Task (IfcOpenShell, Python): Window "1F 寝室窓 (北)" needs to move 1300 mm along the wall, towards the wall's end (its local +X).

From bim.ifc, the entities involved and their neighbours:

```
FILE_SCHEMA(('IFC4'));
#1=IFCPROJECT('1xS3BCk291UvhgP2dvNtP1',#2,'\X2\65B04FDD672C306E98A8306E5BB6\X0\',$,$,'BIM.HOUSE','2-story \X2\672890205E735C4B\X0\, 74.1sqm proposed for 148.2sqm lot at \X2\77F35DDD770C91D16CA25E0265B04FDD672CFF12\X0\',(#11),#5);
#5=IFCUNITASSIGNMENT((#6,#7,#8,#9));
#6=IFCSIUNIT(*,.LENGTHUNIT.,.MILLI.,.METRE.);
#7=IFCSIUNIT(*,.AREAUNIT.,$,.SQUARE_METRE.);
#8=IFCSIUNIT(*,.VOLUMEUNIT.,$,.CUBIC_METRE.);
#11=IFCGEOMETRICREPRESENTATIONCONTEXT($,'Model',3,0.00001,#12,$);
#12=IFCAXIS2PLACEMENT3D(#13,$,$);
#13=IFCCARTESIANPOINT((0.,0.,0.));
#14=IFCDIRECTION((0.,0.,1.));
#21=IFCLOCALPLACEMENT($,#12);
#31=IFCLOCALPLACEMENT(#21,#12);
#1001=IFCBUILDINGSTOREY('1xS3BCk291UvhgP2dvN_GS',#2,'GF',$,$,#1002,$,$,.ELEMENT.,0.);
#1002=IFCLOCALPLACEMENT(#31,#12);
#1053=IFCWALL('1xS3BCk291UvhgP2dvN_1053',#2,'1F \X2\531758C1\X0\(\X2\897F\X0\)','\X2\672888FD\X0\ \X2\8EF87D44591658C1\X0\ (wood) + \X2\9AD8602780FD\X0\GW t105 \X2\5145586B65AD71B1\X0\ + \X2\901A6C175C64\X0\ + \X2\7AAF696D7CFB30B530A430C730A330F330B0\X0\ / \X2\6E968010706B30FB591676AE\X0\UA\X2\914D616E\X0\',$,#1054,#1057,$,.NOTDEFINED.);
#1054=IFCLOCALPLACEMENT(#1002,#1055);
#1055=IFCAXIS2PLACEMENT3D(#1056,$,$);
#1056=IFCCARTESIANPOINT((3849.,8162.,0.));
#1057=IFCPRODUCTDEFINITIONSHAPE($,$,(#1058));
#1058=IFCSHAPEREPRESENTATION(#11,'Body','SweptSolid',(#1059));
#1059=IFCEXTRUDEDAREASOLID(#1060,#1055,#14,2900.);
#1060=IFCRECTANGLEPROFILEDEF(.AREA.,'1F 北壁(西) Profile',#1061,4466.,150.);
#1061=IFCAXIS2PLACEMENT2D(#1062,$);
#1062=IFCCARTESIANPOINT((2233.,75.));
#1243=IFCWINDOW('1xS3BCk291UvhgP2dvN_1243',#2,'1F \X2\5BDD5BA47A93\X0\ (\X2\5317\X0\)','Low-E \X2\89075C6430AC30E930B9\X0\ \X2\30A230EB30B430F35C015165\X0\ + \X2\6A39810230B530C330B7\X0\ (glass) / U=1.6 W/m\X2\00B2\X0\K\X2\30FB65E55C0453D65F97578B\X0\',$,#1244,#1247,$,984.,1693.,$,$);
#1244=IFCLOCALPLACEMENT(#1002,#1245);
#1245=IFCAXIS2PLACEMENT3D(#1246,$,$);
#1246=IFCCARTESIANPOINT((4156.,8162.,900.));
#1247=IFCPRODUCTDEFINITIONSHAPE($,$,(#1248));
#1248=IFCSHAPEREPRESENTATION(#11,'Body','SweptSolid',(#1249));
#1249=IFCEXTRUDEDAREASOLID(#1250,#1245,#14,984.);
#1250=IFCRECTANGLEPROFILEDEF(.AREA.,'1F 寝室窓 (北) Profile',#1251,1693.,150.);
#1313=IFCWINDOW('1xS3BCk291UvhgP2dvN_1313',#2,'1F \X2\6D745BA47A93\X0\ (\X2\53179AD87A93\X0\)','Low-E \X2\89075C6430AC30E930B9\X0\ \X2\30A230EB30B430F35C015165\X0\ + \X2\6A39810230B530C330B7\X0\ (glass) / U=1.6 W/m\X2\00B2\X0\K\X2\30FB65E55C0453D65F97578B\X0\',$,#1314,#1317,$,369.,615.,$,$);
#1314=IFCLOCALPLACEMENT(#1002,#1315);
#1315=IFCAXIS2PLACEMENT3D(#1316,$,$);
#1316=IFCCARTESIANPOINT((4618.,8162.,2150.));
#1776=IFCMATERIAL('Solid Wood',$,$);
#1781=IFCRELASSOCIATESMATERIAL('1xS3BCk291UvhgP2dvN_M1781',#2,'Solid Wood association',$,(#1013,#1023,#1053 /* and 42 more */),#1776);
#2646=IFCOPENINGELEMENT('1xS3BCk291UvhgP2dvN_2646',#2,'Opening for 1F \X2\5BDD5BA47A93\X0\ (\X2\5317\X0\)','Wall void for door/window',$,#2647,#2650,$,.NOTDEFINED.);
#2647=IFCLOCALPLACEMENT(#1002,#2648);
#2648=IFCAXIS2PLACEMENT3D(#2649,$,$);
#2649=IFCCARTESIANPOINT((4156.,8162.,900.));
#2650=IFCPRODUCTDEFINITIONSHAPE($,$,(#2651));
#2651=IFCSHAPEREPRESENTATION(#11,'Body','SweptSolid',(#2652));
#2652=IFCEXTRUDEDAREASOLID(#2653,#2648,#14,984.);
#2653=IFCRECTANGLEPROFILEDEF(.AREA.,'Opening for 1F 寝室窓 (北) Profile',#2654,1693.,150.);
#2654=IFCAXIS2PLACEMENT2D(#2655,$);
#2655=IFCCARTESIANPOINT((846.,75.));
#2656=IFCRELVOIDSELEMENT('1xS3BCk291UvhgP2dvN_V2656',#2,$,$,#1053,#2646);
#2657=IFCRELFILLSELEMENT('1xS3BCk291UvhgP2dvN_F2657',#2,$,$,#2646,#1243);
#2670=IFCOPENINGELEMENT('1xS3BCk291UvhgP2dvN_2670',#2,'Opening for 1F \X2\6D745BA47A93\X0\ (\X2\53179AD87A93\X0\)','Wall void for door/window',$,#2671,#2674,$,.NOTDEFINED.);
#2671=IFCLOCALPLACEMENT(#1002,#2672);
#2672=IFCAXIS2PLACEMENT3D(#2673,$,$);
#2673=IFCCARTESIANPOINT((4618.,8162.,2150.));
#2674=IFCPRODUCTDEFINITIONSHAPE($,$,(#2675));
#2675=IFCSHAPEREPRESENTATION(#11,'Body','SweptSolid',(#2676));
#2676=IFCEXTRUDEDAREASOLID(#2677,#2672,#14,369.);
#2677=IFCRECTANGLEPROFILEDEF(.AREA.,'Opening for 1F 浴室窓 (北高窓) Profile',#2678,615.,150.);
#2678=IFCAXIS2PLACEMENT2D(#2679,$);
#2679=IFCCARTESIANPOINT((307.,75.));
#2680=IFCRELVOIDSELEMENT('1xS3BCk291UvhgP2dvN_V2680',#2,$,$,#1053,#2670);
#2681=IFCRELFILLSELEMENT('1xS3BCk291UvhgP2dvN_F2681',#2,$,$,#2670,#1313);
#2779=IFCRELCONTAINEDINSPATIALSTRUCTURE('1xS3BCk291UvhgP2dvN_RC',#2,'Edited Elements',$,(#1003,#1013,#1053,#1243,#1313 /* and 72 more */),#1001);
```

```python
import ifcopenshell
import ifcopenshell.api.geometry
import ifcopenshell.util.placement

model = ifcopenshell.open("bim.ifc")

window = model.by_guid("1xS3BCk291UvhgP2dvN_1243")
opening = window.FillsVoids[0].RelatingOpeningElement
wall = opening.VoidsElements[0].RelatingBuildingElement

wall_matrix = ifcopenshell.util.placement.get_local_placement(wall.ObjectPlacement)
shift = wall_matrix[:3, 0] * 1300.0
before = ifcopenshell.util.placement.get_local_placement(window.ObjectPlacement)[:3, 3].copy()

# The window is not placed relative to its opening, so move both.
for product in (opening, window):
    matrix = ifcopenshell.util.placement.get_local_placement(product.ObjectPlacement)
    matrix[:3, 3] += shift
    ifcopenshell.api.geometry.edit_object_placement(model, product=product, matrix=matrix, is_si=False)

after = ifcopenshell.util.placement.get_local_placement(window.ObjectPlacement)[:3, 3]
print("window moved by", (after - before).round(3) + 0.0)

model.write("bim-out.ifc")
```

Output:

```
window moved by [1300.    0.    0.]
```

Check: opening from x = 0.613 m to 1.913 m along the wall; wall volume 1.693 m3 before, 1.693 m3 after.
